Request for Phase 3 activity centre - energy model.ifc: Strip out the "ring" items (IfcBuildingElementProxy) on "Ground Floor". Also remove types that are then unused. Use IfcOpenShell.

First a look at what the model holds.

```python
import ifcopenshell
import ifcopenshell.util.element

model = ifcopenshell.open("Phase 3 activity centre - energy model.ifc")
print(model.schema)
storey = next(s for s in model.by_type("IfcBuildingStorey") if s.Name == "Ground Floor")
proxies = [e for e in ifcopenshell.util.element.get_decomposition(storey) if e.is_a("IfcBuildingElementProxy")]
seen = {}
for e in proxies:
    element_type = ifcopenshell.util.element.get_type(e)
    name = element_type.Name if element_type not in (None, e) else None
    seen[name] = seen.get(name, 0) + 1
for name, count in sorted(seen.items(), key=str):
    print(count, "x", name)
```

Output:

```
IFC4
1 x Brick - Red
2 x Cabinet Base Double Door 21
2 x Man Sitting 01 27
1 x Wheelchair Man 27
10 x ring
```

```python
import ifcopenshell
import ifcopenshell.api.root
import ifcopenshell.util.element

model = ifcopenshell.open("Phase 3 activity centre - energy model.ifc")

storey = next(s for s in model.by_type("IfcBuildingStorey") if s.Name == "Ground Floor")
proxies = [e for e in ifcopenshell.util.element.get_decomposition(storey) if e.is_a("IfcBuildingElementProxy")]
targets = [e for e in proxies if (t := ifcopenshell.util.element.get_type(e)) not in (None, e) and t.Name == "ring"]
types = {ifcopenshell.util.element.get_type(e) for e in targets} - {None, *targets}

for e in targets:
    ifcopenshell.api.root.remove_product(model, product=e)
print(len(targets), "removed")

unused = [t for t in types if not ifcopenshell.util.element.get_types(t)]
for t in unused:
    ifcopenshell.api.root.remove_product(model, product=t)
print(len(unused), "unused types removed")

model.write("Phase 3 activity centre - energy model_rev.ifc")
```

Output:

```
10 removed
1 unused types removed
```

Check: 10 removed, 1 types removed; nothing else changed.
